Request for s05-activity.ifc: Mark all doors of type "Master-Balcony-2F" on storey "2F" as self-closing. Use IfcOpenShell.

First a look at what the model holds.

```python
import ifcopenshell
import ifcopenshell.util.element

model = ifcopenshell.open("s05-activity.ifc")
print(model.schema)
storey = next(s for s in model.by_type("IfcBuildingStorey") if s.Name == "2F")
doors = [e for e in ifcopenshell.util.element.get_decomposition(storey) if e.is_a("IfcDoor")]
seen = {}
for e in doors:
    element_type = ifcopenshell.util.element.get_type(e)
    key = (element_type.Name if element_type != e and element_type else None, ifcopenshell.util.element.get_pset(e, "Pset_DoorCommon", "SelfClosing"))
    seen[key] = seen.get(key, 0) + 1
for (name, value), count in sorted(seen.items(), key=str):
    print(count, "x", name, "|", value)
```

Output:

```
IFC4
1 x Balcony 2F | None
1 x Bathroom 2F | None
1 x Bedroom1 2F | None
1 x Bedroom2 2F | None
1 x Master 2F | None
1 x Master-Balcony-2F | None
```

```python
import ifcopenshell
import ifcopenshell.api.pset
import ifcopenshell.util.element

model = ifcopenshell.open("s05-activity.ifc")

storey = next(s for s in model.by_type("IfcBuildingStorey") if s.Name == "2F")
doors = [e for e in ifcopenshell.util.element.get_decomposition(storey) if e.is_a("IfcDoor")]

count = 0
for e in doors:
    element_type = ifcopenshell.util.element.get_type(e)
    if element_type in (None, e) or element_type.Name != "Master-Balcony-2F":
        continue
    # add_pset returns the element's existing set when there is one.
    pset = ifcopenshell.api.pset.add_pset(model, product=e, name="Pset_DoorCommon")
    ifcopenshell.api.pset.edit_pset(model, pset=pset, properties={"SelfClosing": True})
    count += 1

print(count, "doors updated")

model.write("s05-activity_rev.ifc")
```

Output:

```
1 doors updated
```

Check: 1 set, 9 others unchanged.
